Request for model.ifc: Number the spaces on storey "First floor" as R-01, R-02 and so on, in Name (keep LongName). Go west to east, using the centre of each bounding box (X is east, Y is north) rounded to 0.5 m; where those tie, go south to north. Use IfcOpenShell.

First a look at what the model holds.

```python
import ifcopenshell
import ifcopenshell.util.element
import ifcopenshell.util.placement

model = ifcopenshell.open("model.ifc")
print(model.schema)
storey = next(s for s in model.by_type("IfcBuildingStorey") if s.Name == "First floor")
spaces = [e for e in ifcopenshell.util.element.get_decomposition(storey) if e.is_a("IfcSpace")]
for e in sorted(spaces, key=lambda e: e.id()):
    origin = ifcopenshell.util.placement.get_local_placement(e.ObjectPlacement)[:3, 3]
    print(e.id(), e.Name, e.LongName, origin.round(2) + 0.0, sep=" | ")
```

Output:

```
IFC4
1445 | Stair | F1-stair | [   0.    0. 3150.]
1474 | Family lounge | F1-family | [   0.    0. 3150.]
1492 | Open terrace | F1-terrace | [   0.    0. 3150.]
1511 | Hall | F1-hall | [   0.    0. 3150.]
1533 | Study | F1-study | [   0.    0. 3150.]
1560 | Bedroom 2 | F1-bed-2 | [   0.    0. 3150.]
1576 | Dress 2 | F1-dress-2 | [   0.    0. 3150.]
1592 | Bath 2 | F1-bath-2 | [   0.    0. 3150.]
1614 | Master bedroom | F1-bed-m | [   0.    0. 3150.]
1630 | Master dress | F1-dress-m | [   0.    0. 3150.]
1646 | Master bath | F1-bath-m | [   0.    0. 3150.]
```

```python
import ifcopenshell
import ifcopenshell.geom
import ifcopenshell.util.element
import ifcopenshell.util.shape

model = ifcopenshell.open("model.ifc")
settings = ifcopenshell.geom.settings()
settings.set("use-world-coords", True)


def centre(element):
    shape = ifcopenshell.geom.create_shape(settings, element)
    return ifcopenshell.util.shape.get_bbox_centroid(shape.geometry)


storey = next(s for s in model.by_type("IfcBuildingStorey") if s.Name == "First floor")
spaces = [e for e in ifcopenshell.util.element.get_decomposition(storey) if e.is_a("IfcSpace")]

# Insertion points can sit at a corner or the storey origin, so sort by the geometry (in metres).
centres = {e: centre(e) for e in spaces}
spaces.sort(key=lambda e: (round(centres[e][0] / 0.5), centres[e][1]))

for i, e in enumerate(spaces, start=1):
    number = f"R-{i:02d}"
    e.Name = number
    print(e.id(), number)

model.write("model_rev.ifc")
```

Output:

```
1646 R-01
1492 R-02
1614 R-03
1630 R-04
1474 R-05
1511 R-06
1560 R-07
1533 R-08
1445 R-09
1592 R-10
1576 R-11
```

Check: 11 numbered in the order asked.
